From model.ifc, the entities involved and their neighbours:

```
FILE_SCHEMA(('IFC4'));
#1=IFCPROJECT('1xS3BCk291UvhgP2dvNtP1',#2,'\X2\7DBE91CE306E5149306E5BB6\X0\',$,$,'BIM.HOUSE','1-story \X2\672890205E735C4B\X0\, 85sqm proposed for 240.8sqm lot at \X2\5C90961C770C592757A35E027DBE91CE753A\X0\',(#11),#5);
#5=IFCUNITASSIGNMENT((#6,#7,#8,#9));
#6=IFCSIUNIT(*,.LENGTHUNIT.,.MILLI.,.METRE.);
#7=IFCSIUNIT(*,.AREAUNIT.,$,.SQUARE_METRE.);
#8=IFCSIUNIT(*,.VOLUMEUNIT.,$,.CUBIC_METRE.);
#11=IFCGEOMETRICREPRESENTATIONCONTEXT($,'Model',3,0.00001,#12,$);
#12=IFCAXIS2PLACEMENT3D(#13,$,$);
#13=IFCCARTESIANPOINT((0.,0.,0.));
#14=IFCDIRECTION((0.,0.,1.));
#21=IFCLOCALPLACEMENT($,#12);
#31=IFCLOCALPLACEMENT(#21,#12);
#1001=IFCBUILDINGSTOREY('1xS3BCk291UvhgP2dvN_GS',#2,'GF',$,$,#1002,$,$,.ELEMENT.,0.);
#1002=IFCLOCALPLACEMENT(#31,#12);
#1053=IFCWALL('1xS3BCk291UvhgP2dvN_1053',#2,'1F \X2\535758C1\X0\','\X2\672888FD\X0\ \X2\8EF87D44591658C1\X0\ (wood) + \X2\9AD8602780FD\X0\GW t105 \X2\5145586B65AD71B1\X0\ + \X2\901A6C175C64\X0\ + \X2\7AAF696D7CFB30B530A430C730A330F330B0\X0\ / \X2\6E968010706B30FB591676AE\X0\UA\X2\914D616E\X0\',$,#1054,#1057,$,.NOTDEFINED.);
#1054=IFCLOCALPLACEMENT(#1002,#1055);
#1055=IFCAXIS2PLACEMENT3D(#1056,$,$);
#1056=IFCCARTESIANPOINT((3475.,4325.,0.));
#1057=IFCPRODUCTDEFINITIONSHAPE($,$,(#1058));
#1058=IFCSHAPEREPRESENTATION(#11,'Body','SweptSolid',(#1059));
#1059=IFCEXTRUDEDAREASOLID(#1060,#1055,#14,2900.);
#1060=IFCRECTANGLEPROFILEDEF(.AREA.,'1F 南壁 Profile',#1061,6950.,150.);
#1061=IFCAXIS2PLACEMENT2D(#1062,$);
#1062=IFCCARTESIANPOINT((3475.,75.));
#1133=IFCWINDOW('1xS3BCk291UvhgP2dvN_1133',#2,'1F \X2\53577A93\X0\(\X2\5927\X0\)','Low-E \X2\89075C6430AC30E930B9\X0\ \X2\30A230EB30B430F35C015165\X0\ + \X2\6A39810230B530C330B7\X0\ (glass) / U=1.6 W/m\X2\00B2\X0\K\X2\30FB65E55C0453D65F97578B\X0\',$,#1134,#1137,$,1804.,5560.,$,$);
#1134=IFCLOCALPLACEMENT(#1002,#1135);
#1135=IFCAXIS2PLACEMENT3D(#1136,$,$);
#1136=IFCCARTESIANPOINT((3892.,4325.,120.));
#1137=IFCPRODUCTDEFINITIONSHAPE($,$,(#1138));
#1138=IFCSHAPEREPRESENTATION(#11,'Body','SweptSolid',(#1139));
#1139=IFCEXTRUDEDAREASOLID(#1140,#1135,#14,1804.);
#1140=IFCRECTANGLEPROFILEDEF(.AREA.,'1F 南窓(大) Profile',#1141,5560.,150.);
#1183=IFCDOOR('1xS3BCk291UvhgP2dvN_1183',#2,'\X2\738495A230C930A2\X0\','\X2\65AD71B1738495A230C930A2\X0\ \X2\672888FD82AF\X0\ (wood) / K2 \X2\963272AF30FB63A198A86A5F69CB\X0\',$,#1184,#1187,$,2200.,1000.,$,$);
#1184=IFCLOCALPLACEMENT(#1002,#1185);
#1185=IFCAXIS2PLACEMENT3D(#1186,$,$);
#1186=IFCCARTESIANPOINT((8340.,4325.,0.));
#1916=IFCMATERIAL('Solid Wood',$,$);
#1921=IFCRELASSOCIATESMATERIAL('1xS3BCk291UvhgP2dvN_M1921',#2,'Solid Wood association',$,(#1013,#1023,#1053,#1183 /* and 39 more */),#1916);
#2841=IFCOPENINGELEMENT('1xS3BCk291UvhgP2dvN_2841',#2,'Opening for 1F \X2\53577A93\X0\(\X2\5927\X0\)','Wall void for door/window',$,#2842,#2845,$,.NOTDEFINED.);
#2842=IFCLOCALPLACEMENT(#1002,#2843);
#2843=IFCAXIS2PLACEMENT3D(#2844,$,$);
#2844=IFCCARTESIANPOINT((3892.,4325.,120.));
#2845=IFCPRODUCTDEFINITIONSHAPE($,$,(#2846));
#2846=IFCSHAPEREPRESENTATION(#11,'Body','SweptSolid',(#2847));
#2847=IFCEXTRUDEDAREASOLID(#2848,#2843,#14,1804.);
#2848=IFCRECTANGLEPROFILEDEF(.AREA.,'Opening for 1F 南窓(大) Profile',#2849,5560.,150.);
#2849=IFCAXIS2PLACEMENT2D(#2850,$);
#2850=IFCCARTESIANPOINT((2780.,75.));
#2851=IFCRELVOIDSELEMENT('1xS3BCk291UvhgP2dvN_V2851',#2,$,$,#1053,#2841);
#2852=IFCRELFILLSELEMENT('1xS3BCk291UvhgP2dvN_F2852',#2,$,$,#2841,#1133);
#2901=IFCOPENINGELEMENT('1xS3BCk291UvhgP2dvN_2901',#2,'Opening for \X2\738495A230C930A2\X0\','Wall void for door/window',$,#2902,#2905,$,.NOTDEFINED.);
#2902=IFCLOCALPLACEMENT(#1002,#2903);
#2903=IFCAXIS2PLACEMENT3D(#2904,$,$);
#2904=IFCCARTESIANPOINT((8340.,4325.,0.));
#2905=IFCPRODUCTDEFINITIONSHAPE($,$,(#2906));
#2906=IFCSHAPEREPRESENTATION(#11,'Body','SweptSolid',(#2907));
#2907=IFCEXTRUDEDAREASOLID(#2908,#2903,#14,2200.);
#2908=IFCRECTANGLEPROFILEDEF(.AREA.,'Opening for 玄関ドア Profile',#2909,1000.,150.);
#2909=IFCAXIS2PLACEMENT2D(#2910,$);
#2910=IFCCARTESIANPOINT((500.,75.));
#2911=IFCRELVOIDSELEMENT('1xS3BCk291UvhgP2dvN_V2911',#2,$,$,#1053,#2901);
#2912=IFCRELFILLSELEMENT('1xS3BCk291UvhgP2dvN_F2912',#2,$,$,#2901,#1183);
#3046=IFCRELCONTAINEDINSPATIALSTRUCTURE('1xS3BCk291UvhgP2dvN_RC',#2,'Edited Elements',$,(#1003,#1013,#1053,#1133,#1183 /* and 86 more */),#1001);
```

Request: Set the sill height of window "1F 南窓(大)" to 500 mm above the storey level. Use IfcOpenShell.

```python
import numpy as np
import ifcopenshell
import ifcopenshell.api.geometry
import ifcopenshell.geom
import ifcopenshell.util.element
import ifcopenshell.util.placement
import ifcopenshell.util.shape
import ifcopenshell.util.unit

model = ifcopenshell.open("model.ifc")
unit_scale = ifcopenshell.util.unit.calculate_unit_scale(model)

window = model.by_guid("1xS3BCk291UvhgP2dvN_1133")
opening = window.FillsVoids[0].RelatingOpeningElement
storey = ifcopenshell.util.element.get_container(window, ifc_class="IfcBuildingStorey")
level = ifcopenshell.util.placement.get_local_placement(storey.ObjectPlacement)[2, 3]

# The opening's origin need not be at the sill, so measure its lowest point.
shape = ifcopenshell.geom.create_shape(ifcopenshell.geom.settings(), opening)
bottom = ifcopenshell.util.shape.get_shape_bottom_elevation(shape, shape.geometry) / unit_scale
dz = level + 500.0 - bottom

shift = np.array([0.0, 0.0, dz])
# The window is not placed relative to its opening, so move both.
for product in (opening, window):
    matrix = ifcopenshell.util.placement.get_local_placement(product.ObjectPlacement)
    matrix[:3, 3] += shift
    ifcopenshell.api.geometry.edit_object_placement(model, product=product, matrix=matrix, is_si=False)

print(f"moved by {dz * unit_scale:+.3f} m")

model.write("model_edited.ifc")
```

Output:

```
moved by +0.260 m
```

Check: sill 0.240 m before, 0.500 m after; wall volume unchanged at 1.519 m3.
